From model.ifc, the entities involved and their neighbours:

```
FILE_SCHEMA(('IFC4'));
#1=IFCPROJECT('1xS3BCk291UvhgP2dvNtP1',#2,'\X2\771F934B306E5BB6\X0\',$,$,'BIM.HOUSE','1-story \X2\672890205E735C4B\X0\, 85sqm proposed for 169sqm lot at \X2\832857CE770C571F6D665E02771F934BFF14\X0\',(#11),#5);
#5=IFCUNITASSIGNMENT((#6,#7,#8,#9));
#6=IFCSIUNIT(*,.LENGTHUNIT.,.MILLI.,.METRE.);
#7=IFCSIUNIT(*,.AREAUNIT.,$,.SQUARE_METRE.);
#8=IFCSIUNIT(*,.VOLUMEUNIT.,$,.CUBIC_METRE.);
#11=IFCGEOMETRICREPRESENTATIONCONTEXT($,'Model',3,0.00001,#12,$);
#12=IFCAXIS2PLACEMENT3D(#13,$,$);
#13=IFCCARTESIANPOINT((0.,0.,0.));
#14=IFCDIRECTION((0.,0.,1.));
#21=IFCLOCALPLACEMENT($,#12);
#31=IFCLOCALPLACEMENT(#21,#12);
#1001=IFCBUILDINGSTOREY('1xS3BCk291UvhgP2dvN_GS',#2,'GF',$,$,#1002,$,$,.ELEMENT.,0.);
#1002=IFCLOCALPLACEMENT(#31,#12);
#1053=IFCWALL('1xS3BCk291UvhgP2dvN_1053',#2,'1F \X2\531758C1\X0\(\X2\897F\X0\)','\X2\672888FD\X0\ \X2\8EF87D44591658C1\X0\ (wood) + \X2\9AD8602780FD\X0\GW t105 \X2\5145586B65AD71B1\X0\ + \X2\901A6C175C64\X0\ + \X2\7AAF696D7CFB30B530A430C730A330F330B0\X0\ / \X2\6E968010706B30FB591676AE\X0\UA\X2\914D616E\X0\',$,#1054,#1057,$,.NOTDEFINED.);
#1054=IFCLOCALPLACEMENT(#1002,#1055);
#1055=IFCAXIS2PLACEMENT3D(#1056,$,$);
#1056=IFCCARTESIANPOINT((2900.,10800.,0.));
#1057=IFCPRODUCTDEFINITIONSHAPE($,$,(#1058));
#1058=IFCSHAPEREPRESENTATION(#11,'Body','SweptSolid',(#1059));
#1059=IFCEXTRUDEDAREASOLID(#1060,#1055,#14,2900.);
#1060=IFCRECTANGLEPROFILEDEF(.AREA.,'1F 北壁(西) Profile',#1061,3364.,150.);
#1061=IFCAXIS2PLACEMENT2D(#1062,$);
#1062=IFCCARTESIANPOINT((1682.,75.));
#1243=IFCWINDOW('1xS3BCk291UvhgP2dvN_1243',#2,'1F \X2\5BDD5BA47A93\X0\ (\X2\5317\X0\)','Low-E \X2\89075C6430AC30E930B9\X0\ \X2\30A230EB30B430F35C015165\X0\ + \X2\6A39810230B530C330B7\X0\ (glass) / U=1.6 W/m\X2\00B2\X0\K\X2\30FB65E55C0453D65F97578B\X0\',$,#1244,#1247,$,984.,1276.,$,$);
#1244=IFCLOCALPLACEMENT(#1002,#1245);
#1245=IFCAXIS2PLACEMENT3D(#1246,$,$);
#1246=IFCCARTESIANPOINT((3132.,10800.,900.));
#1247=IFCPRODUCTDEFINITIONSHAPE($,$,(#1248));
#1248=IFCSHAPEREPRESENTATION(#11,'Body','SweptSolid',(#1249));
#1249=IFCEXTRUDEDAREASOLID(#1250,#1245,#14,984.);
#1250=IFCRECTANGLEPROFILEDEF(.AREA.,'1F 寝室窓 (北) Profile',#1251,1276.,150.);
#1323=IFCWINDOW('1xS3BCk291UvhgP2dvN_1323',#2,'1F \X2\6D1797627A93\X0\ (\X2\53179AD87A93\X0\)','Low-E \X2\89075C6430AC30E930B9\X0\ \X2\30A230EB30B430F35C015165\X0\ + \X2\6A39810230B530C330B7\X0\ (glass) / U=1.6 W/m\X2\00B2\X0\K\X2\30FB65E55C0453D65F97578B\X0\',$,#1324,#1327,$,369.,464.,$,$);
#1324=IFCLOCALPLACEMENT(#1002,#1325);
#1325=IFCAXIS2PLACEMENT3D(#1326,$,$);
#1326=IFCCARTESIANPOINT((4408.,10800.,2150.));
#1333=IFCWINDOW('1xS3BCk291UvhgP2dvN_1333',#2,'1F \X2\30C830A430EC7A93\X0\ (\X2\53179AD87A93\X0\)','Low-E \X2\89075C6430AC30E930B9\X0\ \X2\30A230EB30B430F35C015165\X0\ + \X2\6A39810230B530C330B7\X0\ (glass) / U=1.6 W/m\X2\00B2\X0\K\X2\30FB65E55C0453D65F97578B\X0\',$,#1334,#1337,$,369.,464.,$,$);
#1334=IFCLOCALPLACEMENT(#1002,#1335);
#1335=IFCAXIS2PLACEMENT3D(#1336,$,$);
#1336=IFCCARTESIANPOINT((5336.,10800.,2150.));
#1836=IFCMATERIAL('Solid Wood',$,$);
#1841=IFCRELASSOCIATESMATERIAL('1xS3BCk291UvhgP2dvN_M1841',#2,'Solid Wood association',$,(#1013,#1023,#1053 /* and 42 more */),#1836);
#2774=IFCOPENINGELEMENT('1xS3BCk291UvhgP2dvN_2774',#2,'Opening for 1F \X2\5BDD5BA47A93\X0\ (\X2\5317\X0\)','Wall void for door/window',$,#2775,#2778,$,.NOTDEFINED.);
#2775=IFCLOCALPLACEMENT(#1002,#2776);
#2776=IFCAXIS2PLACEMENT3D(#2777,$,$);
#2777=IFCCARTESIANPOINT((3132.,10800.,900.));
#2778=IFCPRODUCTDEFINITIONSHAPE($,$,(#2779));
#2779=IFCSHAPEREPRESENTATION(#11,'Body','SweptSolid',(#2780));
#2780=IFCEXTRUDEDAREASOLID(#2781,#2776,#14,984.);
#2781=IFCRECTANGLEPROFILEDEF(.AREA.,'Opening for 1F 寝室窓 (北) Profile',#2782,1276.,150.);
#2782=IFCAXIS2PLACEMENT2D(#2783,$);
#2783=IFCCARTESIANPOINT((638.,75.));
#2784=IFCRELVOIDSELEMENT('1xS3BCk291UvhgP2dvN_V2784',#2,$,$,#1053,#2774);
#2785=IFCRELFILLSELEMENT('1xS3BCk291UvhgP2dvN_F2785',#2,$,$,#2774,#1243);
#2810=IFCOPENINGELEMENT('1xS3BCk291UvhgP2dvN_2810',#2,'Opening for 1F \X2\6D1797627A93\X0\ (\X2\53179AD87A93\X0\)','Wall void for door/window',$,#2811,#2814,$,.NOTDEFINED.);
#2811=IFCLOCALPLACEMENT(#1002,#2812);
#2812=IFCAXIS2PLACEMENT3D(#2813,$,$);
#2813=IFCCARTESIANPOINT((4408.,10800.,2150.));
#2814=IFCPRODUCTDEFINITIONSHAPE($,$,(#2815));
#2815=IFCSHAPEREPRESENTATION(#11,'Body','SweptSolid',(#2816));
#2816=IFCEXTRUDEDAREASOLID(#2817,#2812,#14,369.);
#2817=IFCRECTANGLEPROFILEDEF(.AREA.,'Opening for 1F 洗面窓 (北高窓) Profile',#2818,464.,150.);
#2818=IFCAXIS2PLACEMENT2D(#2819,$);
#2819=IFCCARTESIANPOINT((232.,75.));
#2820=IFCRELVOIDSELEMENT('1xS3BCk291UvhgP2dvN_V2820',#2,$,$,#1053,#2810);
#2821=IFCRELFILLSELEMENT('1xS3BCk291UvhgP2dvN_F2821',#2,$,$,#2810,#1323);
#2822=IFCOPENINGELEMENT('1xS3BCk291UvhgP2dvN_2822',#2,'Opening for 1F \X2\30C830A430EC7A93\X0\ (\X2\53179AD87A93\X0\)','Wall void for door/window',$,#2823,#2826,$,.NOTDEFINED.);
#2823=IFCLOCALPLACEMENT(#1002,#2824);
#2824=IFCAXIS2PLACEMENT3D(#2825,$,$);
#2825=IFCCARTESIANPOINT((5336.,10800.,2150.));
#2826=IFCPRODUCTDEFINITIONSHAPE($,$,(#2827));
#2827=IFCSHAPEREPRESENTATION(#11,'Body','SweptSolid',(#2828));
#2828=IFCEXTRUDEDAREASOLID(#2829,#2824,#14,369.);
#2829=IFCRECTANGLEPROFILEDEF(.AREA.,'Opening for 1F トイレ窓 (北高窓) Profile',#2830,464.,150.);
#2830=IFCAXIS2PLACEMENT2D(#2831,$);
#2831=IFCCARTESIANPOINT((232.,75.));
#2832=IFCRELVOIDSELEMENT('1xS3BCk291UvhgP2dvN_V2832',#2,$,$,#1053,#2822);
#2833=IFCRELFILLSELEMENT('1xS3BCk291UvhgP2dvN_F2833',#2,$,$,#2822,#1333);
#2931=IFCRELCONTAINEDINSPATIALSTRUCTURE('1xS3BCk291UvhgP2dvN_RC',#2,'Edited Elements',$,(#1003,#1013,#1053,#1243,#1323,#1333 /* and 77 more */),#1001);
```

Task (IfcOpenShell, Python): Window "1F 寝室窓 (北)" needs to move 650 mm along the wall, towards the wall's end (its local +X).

```python
import ifcopenshell
import ifcopenshell.api.geometry
import ifcopenshell.util.placement
import ifcopenshell.util.unit

model = ifcopenshell.open("model.ifc")
unit_scale = ifcopenshell.util.unit.calculate_unit_scale(model)

window = model.by_id(1243)
opening = window.FillsVoids[0].RelatingOpeningElement
wall = opening.VoidsElements[0].RelatingBuildingElement

wall_matrix = ifcopenshell.util.placement.get_local_placement(wall.ObjectPlacement)
shift = wall_matrix[:3, 0] * 0.65 / unit_scale
before = ifcopenshell.util.placement.get_local_placement(window.ObjectPlacement)[:3, 3].copy()

# The window is not placed relative to its opening, so move both.
for product in (opening, window):
    matrix = ifcopenshell.util.placement.get_local_placement(product.ObjectPlacement)
    matrix[:3, 3] += shift
    ifcopenshell.api.geometry.edit_object_placement(model, product=product, matrix=matrix, is_si=False)

after = ifcopenshell.util.placement.get_local_placement(window.ObjectPlacement)[:3, 3]
print("window moved by", (after - before).round(3) + 0.0)

model.write("model_rev.ifc")
```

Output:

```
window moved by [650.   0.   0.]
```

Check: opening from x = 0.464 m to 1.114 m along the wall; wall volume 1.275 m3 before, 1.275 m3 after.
